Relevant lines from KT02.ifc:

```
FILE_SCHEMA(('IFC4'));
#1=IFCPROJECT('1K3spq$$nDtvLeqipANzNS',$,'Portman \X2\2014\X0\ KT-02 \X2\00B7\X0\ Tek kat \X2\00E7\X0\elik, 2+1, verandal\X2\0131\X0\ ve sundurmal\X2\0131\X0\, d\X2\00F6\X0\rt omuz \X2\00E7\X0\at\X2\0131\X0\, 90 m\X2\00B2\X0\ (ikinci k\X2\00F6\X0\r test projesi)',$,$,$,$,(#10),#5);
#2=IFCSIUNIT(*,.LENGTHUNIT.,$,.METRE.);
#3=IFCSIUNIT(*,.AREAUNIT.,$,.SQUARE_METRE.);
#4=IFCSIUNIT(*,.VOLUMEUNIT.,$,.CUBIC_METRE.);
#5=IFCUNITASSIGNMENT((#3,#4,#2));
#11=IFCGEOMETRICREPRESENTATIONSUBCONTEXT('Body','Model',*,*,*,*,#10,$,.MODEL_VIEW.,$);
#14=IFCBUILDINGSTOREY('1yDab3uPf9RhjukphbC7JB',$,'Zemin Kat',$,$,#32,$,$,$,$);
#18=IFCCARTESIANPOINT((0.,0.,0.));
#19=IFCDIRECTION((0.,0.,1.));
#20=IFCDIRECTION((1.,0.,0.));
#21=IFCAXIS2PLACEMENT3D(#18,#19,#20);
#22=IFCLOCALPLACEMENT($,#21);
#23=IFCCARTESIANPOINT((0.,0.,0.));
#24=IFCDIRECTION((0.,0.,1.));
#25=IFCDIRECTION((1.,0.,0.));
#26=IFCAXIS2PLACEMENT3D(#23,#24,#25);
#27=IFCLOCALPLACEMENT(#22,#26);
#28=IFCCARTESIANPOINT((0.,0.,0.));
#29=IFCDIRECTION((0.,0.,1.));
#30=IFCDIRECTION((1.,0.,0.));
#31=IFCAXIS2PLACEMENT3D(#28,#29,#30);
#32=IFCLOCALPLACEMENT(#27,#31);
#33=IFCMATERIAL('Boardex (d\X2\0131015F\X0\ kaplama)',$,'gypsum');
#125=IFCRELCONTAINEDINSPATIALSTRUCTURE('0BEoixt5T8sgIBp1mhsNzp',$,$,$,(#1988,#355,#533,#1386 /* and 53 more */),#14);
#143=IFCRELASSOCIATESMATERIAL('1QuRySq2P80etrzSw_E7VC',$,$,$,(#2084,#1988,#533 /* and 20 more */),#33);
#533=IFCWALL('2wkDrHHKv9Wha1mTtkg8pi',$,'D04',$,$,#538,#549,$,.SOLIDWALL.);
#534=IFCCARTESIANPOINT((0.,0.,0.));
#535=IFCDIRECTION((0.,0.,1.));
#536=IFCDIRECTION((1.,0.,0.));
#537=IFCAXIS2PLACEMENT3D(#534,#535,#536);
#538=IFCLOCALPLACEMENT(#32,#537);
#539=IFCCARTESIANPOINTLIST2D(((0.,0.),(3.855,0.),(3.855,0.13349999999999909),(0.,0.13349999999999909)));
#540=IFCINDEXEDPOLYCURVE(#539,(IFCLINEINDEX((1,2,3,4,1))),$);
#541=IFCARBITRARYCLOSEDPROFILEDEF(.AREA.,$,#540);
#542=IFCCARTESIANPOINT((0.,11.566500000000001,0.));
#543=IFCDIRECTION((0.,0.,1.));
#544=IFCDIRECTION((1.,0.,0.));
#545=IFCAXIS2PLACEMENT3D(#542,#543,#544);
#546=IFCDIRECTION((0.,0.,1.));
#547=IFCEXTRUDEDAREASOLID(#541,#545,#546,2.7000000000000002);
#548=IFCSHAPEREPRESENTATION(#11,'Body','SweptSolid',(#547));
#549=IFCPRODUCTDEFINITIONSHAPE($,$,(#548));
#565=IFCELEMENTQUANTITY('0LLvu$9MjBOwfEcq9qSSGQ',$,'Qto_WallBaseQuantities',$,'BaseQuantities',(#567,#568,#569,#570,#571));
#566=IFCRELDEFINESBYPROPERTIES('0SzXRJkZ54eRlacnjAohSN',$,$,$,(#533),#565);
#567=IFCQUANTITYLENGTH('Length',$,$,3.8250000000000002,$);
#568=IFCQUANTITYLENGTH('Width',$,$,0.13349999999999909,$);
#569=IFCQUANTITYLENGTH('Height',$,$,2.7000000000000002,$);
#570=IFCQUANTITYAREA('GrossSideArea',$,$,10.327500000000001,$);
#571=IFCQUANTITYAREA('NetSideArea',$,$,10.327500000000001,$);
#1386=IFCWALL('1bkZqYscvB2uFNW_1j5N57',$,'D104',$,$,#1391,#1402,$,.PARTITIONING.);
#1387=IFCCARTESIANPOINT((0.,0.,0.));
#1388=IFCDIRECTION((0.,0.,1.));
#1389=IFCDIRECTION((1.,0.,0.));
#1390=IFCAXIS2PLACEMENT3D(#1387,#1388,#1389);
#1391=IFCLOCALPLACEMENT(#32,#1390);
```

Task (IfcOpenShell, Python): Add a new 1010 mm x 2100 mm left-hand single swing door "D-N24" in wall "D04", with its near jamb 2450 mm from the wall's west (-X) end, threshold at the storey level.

```python
import numpy as np
import ifcopenshell
import ifcopenshell.api.feature
import ifcopenshell.api.geometry
import ifcopenshell.api.pset
import ifcopenshell.api.root
import ifcopenshell.api.spatial
import ifcopenshell.geom
import ifcopenshell.util.element
import ifcopenshell.util.placement
import ifcopenshell.util.representation
import ifcopenshell.util.shape
import ifcopenshell.util.unit

model = ifcopenshell.open("KT02.ifc")
unit_scale = ifcopenshell.util.unit.calculate_unit_scale(model)
area_scale = ifcopenshell.util.unit.calculate_unit_scale(model, "AREAUNIT")
settings = ifcopenshell.geom.settings()


def volume(element):
    """Net volume in cubic metres, openings subtracted."""
    shape = ifcopenshell.geom.create_shape(settings, element)
    return ifcopenshell.util.shape.get_volume(shape.geometry)


wall = model.by_id(533)
storey = ifcopenshell.util.element.get_container(wall, ifc_class="IfcBuildingStorey")
context = ifcopenshell.util.representation.get_context(model, "Model", "Body", "MODEL_VIEW")
before = volume(wall)

width, height, from_end, sill = 1.01, 2.1, 2.45, 0.0  # metres

# The wall runs along its own X axis, and the end named is its -X end.
wall_shape = ifcopenshell.geom.create_shape(settings, wall)
x, y, z = ifcopenshell.util.shape.get_vertices(wall_shape.geometry).T
start = x.min() + from_end
face, thickness = float(y.min()), float(y.max() - y.min())
wall_matrix = ifcopenshell.util.placement.get_local_placement(wall.ObjectPlacement)
level = ifcopenshell.util.placement.get_local_placement(storey.ObjectPlacement)[2, 3]


def in_wall(x, y):
    """Placement at x, y metres in the wall's axes, at sill height."""
    matrix = wall_matrix.copy()
    matrix[:, 3] = wall_matrix @ np.array([x / unit_scale, y / unit_scale, 0.0, 1.0])
    matrix[2, 3] = level + sill / unit_scale
    return matrix


# Opening: a box that overshoots both wall faces by 50 mm.
opening = ifcopenshell.api.root.create_entity(model, ifc_class="IfcOpeningElement", predefined_type="OPENING")
box = ifcopenshell.api.geometry.add_wall_representation(
    model, context=context, length=width, height=height, thickness=thickness + 0.1
)
ifcopenshell.api.geometry.assign_representation(model, product=opening, representation=box)
ifcopenshell.api.geometry.edit_object_placement(model, product=opening, matrix=in_wall(start, face - 0.05), is_si=False)
ifcopenshell.api.feature.add_feature(model, feature=opening, element=wall)

door = ifcopenshell.api.root.create_entity(model, ifc_class="IfcDoor", name="D-N24", predefined_type="DOOR")
door.OverallWidth, door.OverallHeight = width / unit_scale, height / unit_scale
door.OperationType = "SINGLE_SWING_LEFT"
body = ifcopenshell.api.geometry.add_door_representation(
    model,
    context=context,
    overall_width=door.OverallWidth,
    overall_height=door.OverallHeight,
    operation_type="SINGLE_SWING_LEFT",
    lining_properties={"LiningDepth": thickness / unit_scale, "ThresholdDepth": thickness / unit_scale},
)
ifcopenshell.api.geometry.assign_representation(model, product=door, representation=body)
ifcopenshell.api.spatial.assign_container(model, products=[door], relating_structure=storey)
ifcopenshell.api.feature.add_filling(model, opening=opening, element=door)

# The lining spans the wall, so the door starts at the wall face.
ifcopenshell.api.geometry.edit_object_placement(model, product=door, matrix=in_wall(start, face), is_si=False)

after = volume(wall)

# Update the wall's stored quantities.
qto = model.by_id(ifcopenshell.util.element.get_pset(wall, "Qto_WallBaseQuantities", should_inherit=False)["id"])
ifcopenshell.api.pset.edit_qto(model, qto=qto, properties={"NetSideArea": after / thickness / area_scale})

print(f"wall volume {before:.3f} -> {after:.3f} m3")

model.write("KT02-out.ifc")
```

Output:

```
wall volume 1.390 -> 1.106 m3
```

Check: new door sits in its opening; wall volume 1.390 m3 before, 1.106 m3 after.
